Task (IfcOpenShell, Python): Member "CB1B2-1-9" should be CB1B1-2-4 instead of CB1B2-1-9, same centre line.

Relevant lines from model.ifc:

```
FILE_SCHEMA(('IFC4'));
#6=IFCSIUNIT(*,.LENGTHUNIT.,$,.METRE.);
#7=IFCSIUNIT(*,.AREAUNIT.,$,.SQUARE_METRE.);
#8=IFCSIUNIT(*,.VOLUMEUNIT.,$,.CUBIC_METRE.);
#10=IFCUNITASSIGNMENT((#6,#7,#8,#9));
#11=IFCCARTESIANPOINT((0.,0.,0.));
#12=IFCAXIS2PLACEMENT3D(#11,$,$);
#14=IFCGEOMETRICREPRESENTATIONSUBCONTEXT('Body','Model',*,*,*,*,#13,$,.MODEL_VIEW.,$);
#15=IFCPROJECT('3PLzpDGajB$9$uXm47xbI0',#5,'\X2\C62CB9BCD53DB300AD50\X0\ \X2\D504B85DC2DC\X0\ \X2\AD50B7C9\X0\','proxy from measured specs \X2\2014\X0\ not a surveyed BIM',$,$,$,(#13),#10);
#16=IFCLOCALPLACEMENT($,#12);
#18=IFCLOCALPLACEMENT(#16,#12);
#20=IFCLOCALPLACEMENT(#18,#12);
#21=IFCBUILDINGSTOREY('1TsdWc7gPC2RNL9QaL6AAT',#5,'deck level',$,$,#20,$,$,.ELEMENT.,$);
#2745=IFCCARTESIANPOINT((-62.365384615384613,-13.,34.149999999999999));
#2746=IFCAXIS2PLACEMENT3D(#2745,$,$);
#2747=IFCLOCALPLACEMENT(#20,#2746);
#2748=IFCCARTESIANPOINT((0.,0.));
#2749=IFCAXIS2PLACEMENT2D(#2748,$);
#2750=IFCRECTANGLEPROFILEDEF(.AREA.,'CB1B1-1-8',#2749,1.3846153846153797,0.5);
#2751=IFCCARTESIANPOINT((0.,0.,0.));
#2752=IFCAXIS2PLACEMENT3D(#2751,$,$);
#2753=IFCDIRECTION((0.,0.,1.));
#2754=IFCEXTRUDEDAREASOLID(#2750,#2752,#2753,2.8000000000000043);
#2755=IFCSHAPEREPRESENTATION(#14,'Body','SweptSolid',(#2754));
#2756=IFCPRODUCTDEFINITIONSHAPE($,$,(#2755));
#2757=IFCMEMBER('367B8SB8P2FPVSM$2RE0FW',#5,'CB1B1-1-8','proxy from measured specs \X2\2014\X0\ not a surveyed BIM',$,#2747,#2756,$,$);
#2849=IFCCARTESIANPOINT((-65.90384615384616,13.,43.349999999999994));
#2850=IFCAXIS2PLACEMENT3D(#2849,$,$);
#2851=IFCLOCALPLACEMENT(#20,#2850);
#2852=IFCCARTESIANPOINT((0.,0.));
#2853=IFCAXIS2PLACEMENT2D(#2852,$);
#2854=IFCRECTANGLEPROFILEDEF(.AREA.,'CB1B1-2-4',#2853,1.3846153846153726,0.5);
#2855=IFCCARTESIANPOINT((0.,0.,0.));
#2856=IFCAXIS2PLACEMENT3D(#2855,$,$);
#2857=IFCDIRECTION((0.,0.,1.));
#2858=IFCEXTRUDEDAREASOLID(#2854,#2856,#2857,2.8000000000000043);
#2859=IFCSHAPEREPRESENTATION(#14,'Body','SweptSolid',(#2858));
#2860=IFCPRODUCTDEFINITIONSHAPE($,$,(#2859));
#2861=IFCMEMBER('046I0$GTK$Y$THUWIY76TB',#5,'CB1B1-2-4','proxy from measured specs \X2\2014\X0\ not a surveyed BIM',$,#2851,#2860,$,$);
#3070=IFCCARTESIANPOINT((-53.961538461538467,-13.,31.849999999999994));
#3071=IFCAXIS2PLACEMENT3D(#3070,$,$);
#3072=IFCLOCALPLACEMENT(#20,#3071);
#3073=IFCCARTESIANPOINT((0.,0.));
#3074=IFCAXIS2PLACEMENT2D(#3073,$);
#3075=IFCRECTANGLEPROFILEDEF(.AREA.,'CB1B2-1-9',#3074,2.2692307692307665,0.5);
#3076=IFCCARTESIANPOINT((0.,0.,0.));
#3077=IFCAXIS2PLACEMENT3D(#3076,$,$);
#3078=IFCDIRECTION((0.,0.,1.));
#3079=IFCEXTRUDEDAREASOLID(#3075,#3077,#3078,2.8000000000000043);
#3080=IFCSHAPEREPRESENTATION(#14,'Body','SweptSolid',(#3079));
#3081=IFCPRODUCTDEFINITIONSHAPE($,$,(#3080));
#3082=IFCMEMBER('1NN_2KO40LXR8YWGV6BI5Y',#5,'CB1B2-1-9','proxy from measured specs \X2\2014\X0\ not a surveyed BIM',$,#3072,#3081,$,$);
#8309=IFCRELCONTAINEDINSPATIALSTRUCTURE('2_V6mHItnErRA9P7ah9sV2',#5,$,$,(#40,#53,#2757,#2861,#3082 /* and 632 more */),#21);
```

```python
import ifcopenshell
import ifcopenshell.util.element
import ifcopenshell.util.representation

model = ifcopenshell.open("model.ifc")

member = model.by_guid("1NN_2KO40LXR8YWGV6BI5Y")
source = next(p for p in model.by_type("IfcRectangleProfileDef") if p.ProfileName == "CB1B1-2-4")

body = ifcopenshell.util.representation.get_representation(member, "Model", "Body")
solid = body.Items[0]
old_profile = solid.SweptArea

# Copy the section's sizes but keep this member's own profile position.
profile = ifcopenshell.util.element.copy(model, source)
profile.Position = old_profile.Position
solid.SweptArea = profile
if not model.get_total_inverses(old_profile):
    ifcopenshell.util.element.remove_deep2(model, old_profile)
member.Name = member.Name.replace("CB1B2-1-9", "CB1B1-2-4")

print(solid.SweptArea)

model.write("model_edited.ifc")
```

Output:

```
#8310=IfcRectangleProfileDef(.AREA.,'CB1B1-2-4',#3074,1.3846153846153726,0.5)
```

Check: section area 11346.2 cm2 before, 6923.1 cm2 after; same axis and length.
